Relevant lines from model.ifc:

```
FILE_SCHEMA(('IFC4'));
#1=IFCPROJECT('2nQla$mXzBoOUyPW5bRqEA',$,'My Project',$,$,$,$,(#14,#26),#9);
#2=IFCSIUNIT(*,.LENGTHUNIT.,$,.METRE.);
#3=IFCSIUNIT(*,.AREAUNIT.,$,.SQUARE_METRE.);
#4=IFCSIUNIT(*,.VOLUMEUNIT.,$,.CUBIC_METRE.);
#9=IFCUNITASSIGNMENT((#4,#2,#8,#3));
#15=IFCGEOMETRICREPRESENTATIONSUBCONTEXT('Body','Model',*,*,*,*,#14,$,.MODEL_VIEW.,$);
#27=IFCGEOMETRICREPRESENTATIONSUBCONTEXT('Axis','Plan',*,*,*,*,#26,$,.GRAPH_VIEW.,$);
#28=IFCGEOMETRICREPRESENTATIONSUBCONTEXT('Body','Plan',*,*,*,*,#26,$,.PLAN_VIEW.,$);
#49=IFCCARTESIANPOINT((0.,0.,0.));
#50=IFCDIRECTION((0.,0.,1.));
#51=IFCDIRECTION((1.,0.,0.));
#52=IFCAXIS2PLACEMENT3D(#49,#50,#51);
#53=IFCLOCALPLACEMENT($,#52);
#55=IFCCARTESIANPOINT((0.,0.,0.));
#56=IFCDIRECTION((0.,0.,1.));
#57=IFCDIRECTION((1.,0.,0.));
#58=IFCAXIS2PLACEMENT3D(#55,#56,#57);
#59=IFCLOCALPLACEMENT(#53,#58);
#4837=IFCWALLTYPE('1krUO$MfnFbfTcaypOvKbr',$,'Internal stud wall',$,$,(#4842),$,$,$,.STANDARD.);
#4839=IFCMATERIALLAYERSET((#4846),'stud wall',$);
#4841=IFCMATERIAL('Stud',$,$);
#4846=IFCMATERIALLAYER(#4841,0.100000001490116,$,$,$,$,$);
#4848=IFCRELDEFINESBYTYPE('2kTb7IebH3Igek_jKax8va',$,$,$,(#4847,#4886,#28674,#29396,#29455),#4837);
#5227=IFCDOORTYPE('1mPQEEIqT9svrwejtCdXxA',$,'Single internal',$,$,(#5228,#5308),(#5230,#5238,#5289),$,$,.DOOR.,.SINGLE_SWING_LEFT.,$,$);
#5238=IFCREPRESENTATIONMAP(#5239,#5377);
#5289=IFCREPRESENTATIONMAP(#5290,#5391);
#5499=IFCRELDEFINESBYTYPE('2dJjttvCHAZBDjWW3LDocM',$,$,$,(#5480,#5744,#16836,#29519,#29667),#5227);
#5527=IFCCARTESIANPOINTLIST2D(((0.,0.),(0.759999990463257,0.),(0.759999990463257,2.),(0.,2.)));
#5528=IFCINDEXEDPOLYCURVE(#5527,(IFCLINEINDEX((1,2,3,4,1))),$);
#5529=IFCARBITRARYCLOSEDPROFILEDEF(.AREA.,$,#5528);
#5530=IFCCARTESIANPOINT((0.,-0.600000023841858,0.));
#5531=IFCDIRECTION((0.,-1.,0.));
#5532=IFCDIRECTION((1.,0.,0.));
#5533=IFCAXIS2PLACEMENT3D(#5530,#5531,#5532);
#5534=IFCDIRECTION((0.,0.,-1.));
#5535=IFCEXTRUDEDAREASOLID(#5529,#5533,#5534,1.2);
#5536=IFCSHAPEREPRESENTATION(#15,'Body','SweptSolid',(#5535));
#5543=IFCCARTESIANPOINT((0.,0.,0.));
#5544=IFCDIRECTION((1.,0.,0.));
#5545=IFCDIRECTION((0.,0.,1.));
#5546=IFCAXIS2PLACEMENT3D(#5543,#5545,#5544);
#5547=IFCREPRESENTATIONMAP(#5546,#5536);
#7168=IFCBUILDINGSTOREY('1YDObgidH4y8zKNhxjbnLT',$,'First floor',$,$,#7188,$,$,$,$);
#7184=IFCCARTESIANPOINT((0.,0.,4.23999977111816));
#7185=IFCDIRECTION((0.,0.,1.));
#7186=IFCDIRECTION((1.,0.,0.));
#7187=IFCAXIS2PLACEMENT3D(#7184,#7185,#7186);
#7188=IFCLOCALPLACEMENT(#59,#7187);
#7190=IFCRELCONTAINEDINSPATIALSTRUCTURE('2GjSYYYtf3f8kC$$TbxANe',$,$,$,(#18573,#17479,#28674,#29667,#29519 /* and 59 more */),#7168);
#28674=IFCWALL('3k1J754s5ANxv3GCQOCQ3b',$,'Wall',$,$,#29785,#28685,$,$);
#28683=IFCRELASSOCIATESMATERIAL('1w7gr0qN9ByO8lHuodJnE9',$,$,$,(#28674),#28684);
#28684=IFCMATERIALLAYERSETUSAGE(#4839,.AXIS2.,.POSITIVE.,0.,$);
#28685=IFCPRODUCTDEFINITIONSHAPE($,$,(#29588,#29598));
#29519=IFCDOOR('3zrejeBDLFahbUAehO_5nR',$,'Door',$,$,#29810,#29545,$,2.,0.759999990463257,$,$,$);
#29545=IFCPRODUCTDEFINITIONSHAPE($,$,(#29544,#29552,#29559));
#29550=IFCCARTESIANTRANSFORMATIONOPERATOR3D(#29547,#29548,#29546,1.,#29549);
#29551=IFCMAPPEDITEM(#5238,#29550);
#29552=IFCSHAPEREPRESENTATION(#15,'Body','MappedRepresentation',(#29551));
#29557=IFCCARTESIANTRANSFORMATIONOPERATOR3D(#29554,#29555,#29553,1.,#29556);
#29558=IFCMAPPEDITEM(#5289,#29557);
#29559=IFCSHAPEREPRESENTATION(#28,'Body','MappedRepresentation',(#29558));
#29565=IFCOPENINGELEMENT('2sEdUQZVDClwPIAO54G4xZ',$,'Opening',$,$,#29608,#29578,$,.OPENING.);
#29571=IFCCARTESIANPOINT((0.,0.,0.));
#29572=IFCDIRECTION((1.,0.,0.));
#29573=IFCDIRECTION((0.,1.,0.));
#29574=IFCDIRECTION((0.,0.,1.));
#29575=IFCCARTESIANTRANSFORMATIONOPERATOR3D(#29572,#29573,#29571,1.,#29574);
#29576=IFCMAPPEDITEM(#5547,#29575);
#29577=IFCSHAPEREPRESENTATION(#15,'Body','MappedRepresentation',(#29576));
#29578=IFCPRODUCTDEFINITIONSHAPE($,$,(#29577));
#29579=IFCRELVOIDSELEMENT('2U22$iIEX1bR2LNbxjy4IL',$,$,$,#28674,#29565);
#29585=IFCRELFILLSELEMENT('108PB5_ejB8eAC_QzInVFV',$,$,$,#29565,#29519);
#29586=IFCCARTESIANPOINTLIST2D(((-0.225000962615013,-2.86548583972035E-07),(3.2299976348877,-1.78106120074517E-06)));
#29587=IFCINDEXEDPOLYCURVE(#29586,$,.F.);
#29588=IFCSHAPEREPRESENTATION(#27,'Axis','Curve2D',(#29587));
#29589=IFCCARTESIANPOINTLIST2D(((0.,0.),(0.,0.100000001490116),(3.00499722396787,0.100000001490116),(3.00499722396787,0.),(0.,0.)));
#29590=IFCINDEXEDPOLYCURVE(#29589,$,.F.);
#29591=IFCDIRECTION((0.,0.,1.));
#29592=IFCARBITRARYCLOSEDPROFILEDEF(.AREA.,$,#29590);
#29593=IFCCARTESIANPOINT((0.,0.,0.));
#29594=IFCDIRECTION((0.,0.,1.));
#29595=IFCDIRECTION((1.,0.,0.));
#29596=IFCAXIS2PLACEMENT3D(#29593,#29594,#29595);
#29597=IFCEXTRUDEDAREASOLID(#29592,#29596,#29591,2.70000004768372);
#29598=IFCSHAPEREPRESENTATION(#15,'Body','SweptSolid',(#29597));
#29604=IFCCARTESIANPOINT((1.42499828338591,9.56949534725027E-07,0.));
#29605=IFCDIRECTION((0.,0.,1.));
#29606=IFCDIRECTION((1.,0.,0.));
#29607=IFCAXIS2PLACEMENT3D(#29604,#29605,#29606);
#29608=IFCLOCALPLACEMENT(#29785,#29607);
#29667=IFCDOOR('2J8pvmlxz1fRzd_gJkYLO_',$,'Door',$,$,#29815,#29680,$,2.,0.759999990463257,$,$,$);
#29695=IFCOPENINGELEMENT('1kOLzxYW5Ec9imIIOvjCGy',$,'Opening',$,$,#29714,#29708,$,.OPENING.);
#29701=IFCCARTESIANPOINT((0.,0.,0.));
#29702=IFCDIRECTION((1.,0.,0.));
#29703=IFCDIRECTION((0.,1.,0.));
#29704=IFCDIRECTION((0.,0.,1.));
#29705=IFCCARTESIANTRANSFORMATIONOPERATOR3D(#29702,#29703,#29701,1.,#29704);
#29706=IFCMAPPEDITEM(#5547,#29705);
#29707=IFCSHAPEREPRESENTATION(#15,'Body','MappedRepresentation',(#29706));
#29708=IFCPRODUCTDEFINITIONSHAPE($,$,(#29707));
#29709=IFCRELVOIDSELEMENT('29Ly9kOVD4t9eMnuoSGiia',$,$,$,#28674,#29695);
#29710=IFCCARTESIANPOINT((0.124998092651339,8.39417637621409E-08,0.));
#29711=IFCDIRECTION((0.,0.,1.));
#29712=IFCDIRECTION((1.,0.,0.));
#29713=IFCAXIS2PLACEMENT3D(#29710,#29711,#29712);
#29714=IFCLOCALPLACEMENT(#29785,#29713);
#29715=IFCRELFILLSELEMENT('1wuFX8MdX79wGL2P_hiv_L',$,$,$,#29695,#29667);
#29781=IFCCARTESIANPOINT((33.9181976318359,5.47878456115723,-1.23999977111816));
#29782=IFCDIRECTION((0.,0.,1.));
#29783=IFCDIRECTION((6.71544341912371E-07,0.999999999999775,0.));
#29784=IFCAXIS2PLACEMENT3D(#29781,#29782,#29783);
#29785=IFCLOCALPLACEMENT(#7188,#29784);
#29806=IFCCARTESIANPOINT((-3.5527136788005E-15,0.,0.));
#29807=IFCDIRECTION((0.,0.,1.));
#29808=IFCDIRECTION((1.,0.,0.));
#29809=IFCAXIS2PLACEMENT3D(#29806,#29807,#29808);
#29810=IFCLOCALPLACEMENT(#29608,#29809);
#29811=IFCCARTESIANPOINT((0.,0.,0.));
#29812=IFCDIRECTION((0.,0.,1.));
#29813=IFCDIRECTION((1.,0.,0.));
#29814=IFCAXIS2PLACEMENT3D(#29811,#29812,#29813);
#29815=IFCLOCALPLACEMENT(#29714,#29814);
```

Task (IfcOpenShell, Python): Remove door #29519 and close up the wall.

```python
import ifcopenshell
import ifcopenshell.api.feature
import ifcopenshell.api.root
import ifcopenshell.geom
import ifcopenshell.util.shape

model = ifcopenshell.open("model.ifc")
settings = ifcopenshell.geom.settings()


def volume(element):
    """Net volume in cubic metres, openings subtracted."""
    shape = ifcopenshell.geom.create_shape(settings, element)
    return ifcopenshell.util.shape.get_volume(shape.geometry)


door = model.by_guid("3zrejeBDLFahbUAehO_5nR")
opening = door.FillsVoids[0].RelatingOpeningElement
wall = opening.VoidsElements[0].RelatingBuildingElement
before = volume(wall)

ifcopenshell.api.root.remove_product(model, product=door)
ifcopenshell.api.feature.remove_feature(model, feature=opening)

after = volume(wall)

print(f"wall volume {before:.3f} -> {after:.3f} m3")

model.write("model_rev.ifc")
```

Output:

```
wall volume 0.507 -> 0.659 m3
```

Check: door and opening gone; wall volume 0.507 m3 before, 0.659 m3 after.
